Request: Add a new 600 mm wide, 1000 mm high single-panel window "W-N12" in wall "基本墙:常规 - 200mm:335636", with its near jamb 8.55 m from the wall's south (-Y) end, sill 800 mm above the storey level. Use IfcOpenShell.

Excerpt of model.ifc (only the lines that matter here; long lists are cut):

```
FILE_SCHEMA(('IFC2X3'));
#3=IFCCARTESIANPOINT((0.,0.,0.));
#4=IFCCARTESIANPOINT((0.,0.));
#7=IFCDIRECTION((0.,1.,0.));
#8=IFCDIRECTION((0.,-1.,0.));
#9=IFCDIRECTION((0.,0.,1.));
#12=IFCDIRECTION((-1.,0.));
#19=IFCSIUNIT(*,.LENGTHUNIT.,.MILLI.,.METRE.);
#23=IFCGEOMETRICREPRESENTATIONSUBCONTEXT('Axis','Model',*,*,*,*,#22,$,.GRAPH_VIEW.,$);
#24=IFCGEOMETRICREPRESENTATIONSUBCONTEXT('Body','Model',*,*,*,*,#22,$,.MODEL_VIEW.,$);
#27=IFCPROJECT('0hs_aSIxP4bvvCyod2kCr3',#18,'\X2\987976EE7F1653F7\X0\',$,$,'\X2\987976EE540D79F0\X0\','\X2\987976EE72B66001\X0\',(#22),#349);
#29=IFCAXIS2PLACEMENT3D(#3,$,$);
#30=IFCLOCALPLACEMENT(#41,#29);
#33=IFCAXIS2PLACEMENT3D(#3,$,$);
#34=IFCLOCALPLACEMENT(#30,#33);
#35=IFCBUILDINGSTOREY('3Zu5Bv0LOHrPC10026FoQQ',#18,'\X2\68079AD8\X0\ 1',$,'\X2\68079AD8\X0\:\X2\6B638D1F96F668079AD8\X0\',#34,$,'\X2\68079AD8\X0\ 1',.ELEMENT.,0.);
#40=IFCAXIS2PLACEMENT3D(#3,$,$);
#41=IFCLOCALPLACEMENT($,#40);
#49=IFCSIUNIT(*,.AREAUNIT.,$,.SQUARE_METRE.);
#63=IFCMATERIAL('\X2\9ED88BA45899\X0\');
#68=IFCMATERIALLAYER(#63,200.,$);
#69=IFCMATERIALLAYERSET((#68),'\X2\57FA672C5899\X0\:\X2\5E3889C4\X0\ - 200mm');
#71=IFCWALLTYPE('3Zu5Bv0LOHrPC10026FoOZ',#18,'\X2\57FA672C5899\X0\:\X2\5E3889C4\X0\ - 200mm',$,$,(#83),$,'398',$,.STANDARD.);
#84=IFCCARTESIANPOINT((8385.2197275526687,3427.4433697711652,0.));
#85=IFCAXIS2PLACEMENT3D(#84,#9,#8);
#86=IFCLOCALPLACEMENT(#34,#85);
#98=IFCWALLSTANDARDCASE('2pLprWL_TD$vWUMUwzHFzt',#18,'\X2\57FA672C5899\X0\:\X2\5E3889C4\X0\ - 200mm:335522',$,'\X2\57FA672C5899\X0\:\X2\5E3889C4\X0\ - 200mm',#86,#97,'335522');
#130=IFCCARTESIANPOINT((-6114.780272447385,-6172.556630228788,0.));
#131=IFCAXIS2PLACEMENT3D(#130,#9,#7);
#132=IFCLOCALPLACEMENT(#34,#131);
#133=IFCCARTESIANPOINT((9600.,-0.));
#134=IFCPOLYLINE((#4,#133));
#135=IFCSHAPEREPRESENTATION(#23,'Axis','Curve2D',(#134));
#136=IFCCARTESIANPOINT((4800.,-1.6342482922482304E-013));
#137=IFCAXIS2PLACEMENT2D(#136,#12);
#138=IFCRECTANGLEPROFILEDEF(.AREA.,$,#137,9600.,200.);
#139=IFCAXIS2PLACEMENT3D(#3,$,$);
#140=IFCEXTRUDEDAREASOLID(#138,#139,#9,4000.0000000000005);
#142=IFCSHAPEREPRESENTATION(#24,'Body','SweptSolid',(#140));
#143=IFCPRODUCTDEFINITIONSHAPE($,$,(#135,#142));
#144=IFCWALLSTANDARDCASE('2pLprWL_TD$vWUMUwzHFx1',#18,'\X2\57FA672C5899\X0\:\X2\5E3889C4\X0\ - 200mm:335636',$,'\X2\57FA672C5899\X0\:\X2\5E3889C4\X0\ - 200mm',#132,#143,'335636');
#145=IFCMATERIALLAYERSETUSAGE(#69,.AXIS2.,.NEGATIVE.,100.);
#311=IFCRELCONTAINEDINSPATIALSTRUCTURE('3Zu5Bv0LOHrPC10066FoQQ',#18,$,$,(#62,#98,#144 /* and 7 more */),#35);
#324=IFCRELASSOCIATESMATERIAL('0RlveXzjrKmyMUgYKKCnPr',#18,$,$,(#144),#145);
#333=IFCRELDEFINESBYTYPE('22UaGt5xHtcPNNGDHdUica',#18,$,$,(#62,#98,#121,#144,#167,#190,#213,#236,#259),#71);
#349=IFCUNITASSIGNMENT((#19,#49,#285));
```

```python
import numpy as np
import ifcopenshell
import ifcopenshell.api.feature
import ifcopenshell.api.geometry
import ifcopenshell.api.root
import ifcopenshell.api.spatial
import ifcopenshell.api.type
import ifcopenshell.geom
import ifcopenshell.util.element
import ifcopenshell.util.placement
import ifcopenshell.util.representation
import ifcopenshell.util.shape
import ifcopenshell.util.unit

model = ifcopenshell.open("model.ifc")
unit_scale = ifcopenshell.util.unit.calculate_unit_scale(model)
settings = ifcopenshell.geom.settings()


def volume(element):
    """Net volume in cubic metres, openings subtracted."""
    shape = ifcopenshell.geom.create_shape(settings, element)
    return ifcopenshell.util.shape.get_volume(shape.geometry)


wall = model.by_guid("2pLprWL_TD$vWUMUwzHFx1")
storey = ifcopenshell.util.element.get_container(wall, ifc_class="IfcBuildingStorey")
context = ifcopenshell.util.representation.get_context(model, "Model", "Body", "MODEL_VIEW")
before = volume(wall)

width, height, from_end, sill = 0.6, 1, 8.55, 0.8  # metres

# The wall runs along its own X axis, and the end named is its -X end.
wall_shape = ifcopenshell.geom.create_shape(settings, wall)
x, y, z = ifcopenshell.util.shape.get_vertices(wall_shape.geometry).T
start = x.min() + from_end
face, thickness = float(y.min()), float(y.max() - y.min())
wall_matrix = ifcopenshell.util.placement.get_local_placement(wall.ObjectPlacement)
level = ifcopenshell.util.placement.get_local_placement(storey.ObjectPlacement)[2, 3]


def in_wall(x, y):
    """Placement at x, y metres in the wall's axes, at sill height."""
    matrix = wall_matrix.copy()
    matrix[:, 3] = wall_matrix @ np.array([x / unit_scale, y / unit_scale, 0.0, 1.0])
    matrix[2, 3] = level + sill / unit_scale
    return matrix


# Opening: a box that overshoots both wall faces by 50 mm.
opening = ifcopenshell.api.root.create_entity(model, ifc_class="IfcOpeningElement")
box = ifcopenshell.api.geometry.add_wall_representation(
    model, context=context, length=width, height=height, thickness=thickness + 0.1
)
ifcopenshell.api.geometry.assign_representation(model, product=opening, representation=box)
ifcopenshell.api.geometry.edit_object_placement(model, product=opening, matrix=in_wall(start, face - 0.05), is_si=False)
ifcopenshell.api.feature.add_feature(model, feature=opening, element=wall)

window = ifcopenshell.api.root.create_entity(model, ifc_class="IfcWindow", name="W-N12")
window.OverallWidth, window.OverallHeight = width / unit_scale, height / unit_scale
body = ifcopenshell.api.geometry.add_window_representation(
    model,
    context=context,
    overall_width=window.OverallWidth,
    overall_height=window.OverallHeight,
    partition_type="SINGLE_PANEL",
)
ifcopenshell.api.geometry.assign_representation(model, product=window, representation=body)
ifcopenshell.api.spatial.assign_container(model, products=[window], relating_structure=storey)
fills = ifcopenshell.api.feature.add_filling(model, opening=opening, element=window)
fills.OwnerHistory = window.OwnerHistory  # required in IFC2X3

# IFC2X3 keeps the operation on the window style.
style = ifcopenshell.api.root.create_entity(model, ifc_class="IfcWindowStyle", name="W-N12")
style.OperationType, style.ConstructionType = "SINGLE_PANEL", "NOTDEFINED"
style.ParameterTakesPrecedence = style.Sizeable = False
ifcopenshell.api.type.assign_type(model, related_objects=[window], relating_type=style)

# Centre the window in the wall's thickness.
ifcopenshell.api.geometry.edit_object_placement(model, product=window, matrix=in_wall(start, face), is_si=False)
window_shape = ifcopenshell.geom.create_shape(settings, window)
depth = ifcopenshell.util.shape.get_vertices(window_shape.geometry)[:, 1]
offset = face + thickness / 2 - (depth.min() + depth.max()) / 2
ifcopenshell.api.geometry.edit_object_placement(model, product=window, matrix=in_wall(start, offset), is_si=False)

after = volume(wall)

print(f"wall volume {before:.3f} -> {after:.3f} m3")

model.write("model-out.ifc")
```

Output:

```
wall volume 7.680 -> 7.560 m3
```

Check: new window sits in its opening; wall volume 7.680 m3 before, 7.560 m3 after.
